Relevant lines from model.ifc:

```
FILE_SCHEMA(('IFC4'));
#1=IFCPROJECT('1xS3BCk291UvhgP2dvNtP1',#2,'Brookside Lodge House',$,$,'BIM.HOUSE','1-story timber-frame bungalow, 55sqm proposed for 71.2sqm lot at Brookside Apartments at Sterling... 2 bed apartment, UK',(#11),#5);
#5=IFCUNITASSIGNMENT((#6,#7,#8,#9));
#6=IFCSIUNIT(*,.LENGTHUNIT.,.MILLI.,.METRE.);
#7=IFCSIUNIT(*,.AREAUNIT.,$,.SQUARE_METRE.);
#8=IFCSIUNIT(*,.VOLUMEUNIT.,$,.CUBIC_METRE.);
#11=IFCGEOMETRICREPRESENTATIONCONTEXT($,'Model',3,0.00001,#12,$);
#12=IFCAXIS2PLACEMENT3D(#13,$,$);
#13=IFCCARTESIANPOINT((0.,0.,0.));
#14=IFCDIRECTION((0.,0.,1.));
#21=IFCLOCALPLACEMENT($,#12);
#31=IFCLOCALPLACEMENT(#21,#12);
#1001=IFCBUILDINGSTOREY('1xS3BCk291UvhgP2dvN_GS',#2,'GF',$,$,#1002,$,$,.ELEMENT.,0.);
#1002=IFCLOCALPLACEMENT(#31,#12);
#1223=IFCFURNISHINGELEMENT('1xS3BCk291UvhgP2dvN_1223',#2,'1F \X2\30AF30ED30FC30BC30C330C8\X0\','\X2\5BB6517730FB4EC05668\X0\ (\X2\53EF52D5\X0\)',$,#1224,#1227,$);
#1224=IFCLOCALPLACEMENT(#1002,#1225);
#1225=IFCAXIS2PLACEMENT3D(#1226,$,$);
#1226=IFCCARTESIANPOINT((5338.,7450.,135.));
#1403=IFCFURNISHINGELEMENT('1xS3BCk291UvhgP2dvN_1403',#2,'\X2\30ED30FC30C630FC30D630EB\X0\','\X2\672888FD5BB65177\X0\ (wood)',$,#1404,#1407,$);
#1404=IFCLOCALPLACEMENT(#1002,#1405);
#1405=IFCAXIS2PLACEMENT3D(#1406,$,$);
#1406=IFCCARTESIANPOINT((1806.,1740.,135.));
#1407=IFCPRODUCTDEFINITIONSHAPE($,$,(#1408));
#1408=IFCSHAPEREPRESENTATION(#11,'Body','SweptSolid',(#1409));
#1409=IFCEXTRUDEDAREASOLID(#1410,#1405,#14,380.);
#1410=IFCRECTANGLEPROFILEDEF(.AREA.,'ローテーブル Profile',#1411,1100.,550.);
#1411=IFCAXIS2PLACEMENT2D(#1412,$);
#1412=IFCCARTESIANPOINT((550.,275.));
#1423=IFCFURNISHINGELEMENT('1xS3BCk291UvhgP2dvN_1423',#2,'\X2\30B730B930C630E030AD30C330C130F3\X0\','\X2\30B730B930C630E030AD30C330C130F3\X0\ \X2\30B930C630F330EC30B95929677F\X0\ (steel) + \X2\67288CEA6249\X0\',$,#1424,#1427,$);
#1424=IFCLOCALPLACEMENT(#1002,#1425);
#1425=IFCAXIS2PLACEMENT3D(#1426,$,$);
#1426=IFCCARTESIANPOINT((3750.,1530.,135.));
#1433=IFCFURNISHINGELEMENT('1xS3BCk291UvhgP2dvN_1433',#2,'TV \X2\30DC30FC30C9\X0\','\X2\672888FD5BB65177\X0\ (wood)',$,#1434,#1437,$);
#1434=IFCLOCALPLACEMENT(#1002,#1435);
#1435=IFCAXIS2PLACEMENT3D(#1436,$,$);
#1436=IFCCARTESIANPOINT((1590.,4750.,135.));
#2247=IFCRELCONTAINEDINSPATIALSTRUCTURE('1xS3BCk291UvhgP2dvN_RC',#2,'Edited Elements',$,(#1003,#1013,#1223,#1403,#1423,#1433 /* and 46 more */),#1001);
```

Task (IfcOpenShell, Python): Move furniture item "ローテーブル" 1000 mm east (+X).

```python
import ifcopenshell
import ifcopenshell.api.geometry
import ifcopenshell.util.placement
import ifcopenshell.util.unit

model = ifcopenshell.open("model.ifc")
unit_scale = ifcopenshell.util.unit.calculate_unit_scale(model)

item = model.by_guid("1xS3BCk291UvhgP2dvN_1403")
matrix = ifcopenshell.util.placement.get_local_placement(item.ObjectPlacement)
matrix[0, 3] += 1 / unit_scale
ifcopenshell.api.geometry.edit_object_placement(model, product=item, matrix=matrix, is_si=False)

print(ifcopenshell.util.placement.get_local_placement(item.ObjectPlacement).round(3) + 0.0)

model.write("model-out.ifc")
```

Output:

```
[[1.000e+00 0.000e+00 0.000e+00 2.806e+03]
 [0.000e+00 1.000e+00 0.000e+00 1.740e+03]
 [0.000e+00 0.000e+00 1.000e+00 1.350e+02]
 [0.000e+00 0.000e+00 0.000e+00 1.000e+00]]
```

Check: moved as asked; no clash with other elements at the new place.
